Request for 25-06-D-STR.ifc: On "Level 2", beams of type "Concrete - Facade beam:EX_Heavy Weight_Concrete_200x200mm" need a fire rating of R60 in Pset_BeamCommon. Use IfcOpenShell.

First a look at what the model holds.

```python
import ifcopenshell
import ifcopenshell.util.element

model = ifcopenshell.open("25-06-D-STR.ifc")
print(model.schema)
storey = next(s for s in model.by_type("IfcBuildingStorey") if s.Name == "Level 2")
beams = [e for e in ifcopenshell.util.element.get_decomposition(storey) if e.is_a("IfcBeam")]
seen = {}
for e in beams:
    element_type = ifcopenshell.util.element.get_type(e)
    key = (element_type.Name if element_type != e and element_type else None, ifcopenshell.util.element.get_pset(e, "Pset_BeamCommon", "FireRating"))
    seen[key] = seen.get(key, 0) + 1
for (name, value), count in sorted(seen.items(), key=str):
    print(count, "x", name, "|", value)
```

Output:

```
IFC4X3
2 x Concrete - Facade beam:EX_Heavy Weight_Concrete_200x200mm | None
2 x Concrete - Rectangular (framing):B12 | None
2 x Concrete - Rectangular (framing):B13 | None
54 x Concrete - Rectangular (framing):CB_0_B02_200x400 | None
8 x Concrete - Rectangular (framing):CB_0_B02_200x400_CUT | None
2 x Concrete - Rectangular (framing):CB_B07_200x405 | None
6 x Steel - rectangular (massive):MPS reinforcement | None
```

```python
import ifcopenshell
import ifcopenshell.api.pset
import ifcopenshell.util.element

model = ifcopenshell.open("25-06-D-STR.ifc")

storey = next(s for s in model.by_type("IfcBuildingStorey") if s.Name == "Level 2")
beams = [e for e in ifcopenshell.util.element.get_decomposition(storey) if e.is_a("IfcBeam")]

count = 0
for e in beams:
    element_type = ifcopenshell.util.element.get_type(e)
    if element_type in (None, e) or element_type.Name != "Concrete - Facade beam:EX_Heavy Weight_Concrete_200x200mm":
        continue
    # add_pset returns the element's existing set when there is one.
    pset = ifcopenshell.api.pset.add_pset(model, product=e, name="Pset_BeamCommon")
    ifcopenshell.api.pset.edit_pset(model, pset=pset, properties={"FireRating": "R60"})
    count += 1

print(count, "beams updated")

model.write("25-06-D-STR_v2.ifc")
```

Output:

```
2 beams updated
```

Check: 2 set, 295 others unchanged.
